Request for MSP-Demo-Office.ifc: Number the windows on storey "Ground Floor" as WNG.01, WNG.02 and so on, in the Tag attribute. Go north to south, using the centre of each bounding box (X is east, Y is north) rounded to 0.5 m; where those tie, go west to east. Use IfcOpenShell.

First a look at what the model holds.

```python
import ifcopenshell
import ifcopenshell.util.element
import ifcopenshell.util.placement

model = ifcopenshell.open("MSP-Demo-Office.ifc")
print(model.schema)
storey = next(s for s in model.by_type("IfcBuildingStorey") if s.Name == "Ground Floor")
windows = [e for e in ifcopenshell.util.element.get_decomposition(storey) if e.is_a("IfcWindow")]
for e in sorted(windows, key=lambda e: e.id()):
    origin = ifcopenshell.util.placement.get_local_placement(e.ObjectPlacement)[:3, 3]
    print(e.id(), e.Tag, e.Name, origin.round(2) + 0.0, sep=" | ")
```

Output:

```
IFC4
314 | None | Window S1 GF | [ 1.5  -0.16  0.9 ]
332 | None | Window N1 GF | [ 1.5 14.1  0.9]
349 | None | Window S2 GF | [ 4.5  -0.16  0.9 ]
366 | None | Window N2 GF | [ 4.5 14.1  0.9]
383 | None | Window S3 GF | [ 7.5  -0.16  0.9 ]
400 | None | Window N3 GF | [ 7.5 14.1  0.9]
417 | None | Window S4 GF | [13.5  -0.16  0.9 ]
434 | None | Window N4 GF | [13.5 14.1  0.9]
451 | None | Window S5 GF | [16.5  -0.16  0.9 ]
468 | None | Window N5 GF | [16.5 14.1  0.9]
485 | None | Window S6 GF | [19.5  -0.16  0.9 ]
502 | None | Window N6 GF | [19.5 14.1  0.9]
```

```python
import ifcopenshell
import ifcopenshell.geom
import ifcopenshell.util.element
import ifcopenshell.util.shape

model = ifcopenshell.open("MSP-Demo-Office.ifc")
settings = ifcopenshell.geom.settings()
settings.set("use-world-coords", True)


def centre(element):
    shape = ifcopenshell.geom.create_shape(settings, element)
    return ifcopenshell.util.shape.get_bbox_centroid(shape.geometry)


storey = next(s for s in model.by_type("IfcBuildingStorey") if s.Name == "Ground Floor")
windows = [e for e in ifcopenshell.util.element.get_decomposition(storey) if e.is_a("IfcWindow")]

# Insertion points can sit at a corner or the storey origin, so sort by the geometry (in metres).
centres = {e: centre(e) for e in windows}
windows.sort(key=lambda e: (-round(centres[e][1] / 0.5), centres[e][0]))

for i, e in enumerate(windows, start=1):
    number = f"WNG.{i:02d}"
    e.Tag = number
    print(e.id(), number)

model.write("MSP-Demo-Office_rev.ifc")
```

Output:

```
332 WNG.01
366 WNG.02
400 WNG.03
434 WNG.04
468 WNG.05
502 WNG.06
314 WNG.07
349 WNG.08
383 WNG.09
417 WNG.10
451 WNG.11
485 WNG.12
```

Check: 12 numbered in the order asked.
